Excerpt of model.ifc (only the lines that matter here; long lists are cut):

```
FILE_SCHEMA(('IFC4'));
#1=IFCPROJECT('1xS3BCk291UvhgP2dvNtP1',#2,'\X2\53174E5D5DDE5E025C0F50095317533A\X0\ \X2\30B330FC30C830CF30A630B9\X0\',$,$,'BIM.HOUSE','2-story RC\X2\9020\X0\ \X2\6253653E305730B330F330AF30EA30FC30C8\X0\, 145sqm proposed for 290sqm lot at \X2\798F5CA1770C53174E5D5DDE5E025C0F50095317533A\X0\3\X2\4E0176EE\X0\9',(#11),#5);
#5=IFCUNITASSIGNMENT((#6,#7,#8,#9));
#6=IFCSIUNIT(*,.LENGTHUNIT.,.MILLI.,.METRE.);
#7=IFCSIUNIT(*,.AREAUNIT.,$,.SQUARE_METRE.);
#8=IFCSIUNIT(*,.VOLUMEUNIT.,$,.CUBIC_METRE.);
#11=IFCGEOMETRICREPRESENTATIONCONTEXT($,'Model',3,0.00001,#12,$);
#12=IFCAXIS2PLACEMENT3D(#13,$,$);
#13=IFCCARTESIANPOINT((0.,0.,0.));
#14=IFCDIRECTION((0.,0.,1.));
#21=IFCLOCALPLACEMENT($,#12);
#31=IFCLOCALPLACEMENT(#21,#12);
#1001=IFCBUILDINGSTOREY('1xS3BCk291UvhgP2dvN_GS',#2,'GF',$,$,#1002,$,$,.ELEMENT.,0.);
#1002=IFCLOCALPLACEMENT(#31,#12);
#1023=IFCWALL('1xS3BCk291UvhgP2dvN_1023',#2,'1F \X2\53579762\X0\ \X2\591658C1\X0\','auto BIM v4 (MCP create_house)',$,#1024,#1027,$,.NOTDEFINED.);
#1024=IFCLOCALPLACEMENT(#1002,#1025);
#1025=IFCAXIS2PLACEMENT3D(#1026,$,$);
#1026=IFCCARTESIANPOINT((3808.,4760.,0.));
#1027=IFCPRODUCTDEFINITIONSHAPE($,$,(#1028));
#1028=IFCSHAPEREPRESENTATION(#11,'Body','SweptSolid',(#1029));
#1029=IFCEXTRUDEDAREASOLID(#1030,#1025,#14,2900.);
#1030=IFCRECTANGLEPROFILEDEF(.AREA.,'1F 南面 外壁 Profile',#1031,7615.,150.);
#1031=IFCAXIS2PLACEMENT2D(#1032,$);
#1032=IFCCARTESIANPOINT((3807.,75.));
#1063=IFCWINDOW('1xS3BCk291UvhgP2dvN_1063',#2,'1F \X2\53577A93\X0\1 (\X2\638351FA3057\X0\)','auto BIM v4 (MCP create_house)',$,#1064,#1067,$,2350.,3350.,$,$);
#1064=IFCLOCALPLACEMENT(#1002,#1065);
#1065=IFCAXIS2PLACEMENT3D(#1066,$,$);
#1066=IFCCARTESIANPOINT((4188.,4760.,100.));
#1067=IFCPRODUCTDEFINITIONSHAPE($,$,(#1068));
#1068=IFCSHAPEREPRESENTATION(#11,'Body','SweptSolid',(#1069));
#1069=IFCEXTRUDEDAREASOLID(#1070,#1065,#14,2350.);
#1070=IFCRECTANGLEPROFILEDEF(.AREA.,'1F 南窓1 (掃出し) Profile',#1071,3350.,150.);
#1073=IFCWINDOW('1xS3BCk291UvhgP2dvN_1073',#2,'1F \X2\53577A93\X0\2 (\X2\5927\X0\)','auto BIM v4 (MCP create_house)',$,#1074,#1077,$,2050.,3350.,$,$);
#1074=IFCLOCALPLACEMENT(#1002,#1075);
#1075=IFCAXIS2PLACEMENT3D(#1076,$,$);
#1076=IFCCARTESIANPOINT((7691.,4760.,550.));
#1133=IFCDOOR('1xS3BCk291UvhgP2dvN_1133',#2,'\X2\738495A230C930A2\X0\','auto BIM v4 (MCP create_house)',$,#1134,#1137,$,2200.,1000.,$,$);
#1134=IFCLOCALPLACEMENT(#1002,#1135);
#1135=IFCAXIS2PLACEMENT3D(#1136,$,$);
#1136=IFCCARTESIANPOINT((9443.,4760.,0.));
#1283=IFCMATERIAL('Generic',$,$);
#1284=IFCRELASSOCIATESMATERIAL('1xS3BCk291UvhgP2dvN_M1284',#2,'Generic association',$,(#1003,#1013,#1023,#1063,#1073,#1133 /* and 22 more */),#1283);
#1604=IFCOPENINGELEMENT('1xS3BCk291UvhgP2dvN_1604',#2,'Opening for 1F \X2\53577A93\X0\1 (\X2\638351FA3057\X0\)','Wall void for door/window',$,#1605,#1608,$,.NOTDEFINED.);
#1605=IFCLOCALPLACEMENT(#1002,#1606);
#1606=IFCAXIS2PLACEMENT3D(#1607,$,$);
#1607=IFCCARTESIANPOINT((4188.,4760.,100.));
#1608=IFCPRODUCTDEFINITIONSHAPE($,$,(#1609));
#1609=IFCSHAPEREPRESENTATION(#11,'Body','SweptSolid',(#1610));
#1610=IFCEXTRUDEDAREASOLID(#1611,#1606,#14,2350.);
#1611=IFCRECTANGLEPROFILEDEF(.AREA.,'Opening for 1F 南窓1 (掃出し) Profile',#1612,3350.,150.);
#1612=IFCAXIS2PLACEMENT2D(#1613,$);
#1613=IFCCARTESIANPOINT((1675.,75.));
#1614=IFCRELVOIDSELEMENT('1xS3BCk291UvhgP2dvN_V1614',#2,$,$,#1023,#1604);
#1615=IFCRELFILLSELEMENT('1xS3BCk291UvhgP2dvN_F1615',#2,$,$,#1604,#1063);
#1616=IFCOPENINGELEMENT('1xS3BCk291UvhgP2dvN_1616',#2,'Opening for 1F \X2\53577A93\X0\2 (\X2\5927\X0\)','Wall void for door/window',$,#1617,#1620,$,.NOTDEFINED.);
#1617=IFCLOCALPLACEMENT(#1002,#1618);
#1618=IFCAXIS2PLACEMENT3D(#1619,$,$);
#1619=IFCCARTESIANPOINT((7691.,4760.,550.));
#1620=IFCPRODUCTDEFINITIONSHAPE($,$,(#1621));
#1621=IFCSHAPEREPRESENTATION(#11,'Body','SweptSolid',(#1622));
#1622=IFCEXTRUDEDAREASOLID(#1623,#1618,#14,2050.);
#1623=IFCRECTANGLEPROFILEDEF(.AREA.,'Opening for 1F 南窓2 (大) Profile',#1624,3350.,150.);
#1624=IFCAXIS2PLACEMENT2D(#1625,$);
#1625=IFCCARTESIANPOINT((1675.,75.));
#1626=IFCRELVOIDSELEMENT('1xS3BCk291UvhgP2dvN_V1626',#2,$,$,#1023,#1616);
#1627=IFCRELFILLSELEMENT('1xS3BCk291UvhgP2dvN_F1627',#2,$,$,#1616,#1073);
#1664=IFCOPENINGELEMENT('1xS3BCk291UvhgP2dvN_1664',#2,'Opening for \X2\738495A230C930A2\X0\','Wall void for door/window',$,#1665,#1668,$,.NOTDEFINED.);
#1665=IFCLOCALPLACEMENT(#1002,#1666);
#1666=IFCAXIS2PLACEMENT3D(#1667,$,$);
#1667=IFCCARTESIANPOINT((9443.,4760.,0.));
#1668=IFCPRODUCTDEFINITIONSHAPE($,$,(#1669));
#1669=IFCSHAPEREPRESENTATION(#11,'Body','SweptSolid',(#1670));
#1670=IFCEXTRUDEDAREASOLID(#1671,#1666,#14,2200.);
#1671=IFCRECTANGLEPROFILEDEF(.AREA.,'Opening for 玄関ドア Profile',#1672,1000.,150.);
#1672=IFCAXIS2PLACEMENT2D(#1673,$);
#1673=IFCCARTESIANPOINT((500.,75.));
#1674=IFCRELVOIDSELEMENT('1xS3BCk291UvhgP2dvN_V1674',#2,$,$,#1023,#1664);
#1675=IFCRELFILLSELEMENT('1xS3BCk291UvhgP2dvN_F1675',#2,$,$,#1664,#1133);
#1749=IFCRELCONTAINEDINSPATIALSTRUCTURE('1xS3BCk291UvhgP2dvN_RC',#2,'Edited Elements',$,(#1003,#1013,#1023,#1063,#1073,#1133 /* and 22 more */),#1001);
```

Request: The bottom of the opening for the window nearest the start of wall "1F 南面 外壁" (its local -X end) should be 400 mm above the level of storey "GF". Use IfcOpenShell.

```python
import numpy as np
import ifcopenshell
import ifcopenshell.api.geometry
import ifcopenshell.geom
import ifcopenshell.util.element
import ifcopenshell.util.placement
import ifcopenshell.util.shape
import ifcopenshell.util.unit

model = ifcopenshell.open("model.ifc")
unit_scale = ifcopenshell.util.unit.calculate_unit_scale(model)

window = model.by_guid("1xS3BCk291UvhgP2dvN_1063")
opening = window.FillsVoids[0].RelatingOpeningElement
storey = ifcopenshell.util.element.get_container(window, ifc_class="IfcBuildingStorey")
level = ifcopenshell.util.placement.get_local_placement(storey.ObjectPlacement)[2, 3]

# The opening's origin need not be at the sill, so measure its lowest point.
shape = ifcopenshell.geom.create_shape(ifcopenshell.geom.settings(), opening)
bottom = ifcopenshell.util.shape.get_shape_bottom_elevation(shape, shape.geometry) / unit_scale
dz = level + 400.0 - bottom

shift = np.array([0.0, 0.0, dz])
# The window is not placed relative to its opening, so move both.
for product in (opening, window):
    matrix = ifcopenshell.util.placement.get_local_placement(product.ObjectPlacement)
    matrix[:3, 3] += shift
    ifcopenshell.api.geometry.edit_object_placement(model, product=product, matrix=matrix, is_si=False)

print(f"moved by {dz * unit_scale:+.3f} m")

model.write("model_edited.ifc")
```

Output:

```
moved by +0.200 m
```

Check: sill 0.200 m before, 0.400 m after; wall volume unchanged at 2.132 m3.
